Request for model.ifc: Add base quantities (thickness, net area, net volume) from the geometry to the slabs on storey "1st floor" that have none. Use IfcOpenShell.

First a look at what the model holds.

```python
import ifcopenshell
import ifcopenshell.util.element
import ifcopenshell.util.unit

model = ifcopenshell.open("model.ifc")
print(model.schema)
for unit_type in ("LENGTHUNIT", "AREAUNIT", "VOLUMEUNIT"):
    print(unit_type, ifcopenshell.util.unit.calculate_unit_scale(model, unit_type))
storey = next(s for s in model.by_type("IfcBuildingStorey") if s.Name == "1st floor")
slabs = [e for e in ifcopenshell.util.element.get_decomposition(storey) if e.is_a("IfcSlab")]
for e in sorted(slabs, key=lambda e: e.id()):
    print(e.id(), e.is_a(), e.Name, list(ifcopenshell.util.element.get_psets(e, qtos_only=True)), sep=" | ")
```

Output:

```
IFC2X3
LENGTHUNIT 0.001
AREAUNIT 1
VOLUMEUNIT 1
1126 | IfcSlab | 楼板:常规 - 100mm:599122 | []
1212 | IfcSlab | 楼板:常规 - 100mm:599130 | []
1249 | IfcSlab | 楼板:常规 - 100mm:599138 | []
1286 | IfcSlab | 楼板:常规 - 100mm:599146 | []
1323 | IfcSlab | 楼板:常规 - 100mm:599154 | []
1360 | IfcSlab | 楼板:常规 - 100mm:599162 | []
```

```python
import ifcopenshell
import ifcopenshell.api.pset
import ifcopenshell.geom
import ifcopenshell.util.element
import ifcopenshell.util.shape
import ifcopenshell.util.unit

model = ifcopenshell.open("model.ifc")
unit_scale = ifcopenshell.util.unit.calculate_unit_scale(model)
area_scale = ifcopenshell.util.unit.calculate_unit_scale(model, "AREAUNIT")
volume_scale = ifcopenshell.util.unit.calculate_unit_scale(model, "VOLUMEUNIT")
settings = ifcopenshell.geom.settings()

storey = next(s for s in model.by_type("IfcBuildingStorey") if s.Name == "1st floor")
slabs = [e for e in ifcopenshell.util.element.get_decomposition(storey) if e.is_a("IfcSlab")]

for e in sorted(slabs, key=lambda e: e.id()):
    if ifcopenshell.util.element.get_psets(e, qtos_only=True, should_inherit=False):
        continue
    # Geometry comes back in metres, in the element's own axes.
    shape = ifcopenshell.geom.create_shape(settings, e)
    values = {
        "Width": ifcopenshell.util.shape.get_z(shape.geometry) / unit_scale,
        "NetArea": ifcopenshell.util.shape.get_footprint_area(shape.geometry) / area_scale,
        "NetVolume": ifcopenshell.util.shape.get_volume(shape.geometry) / volume_scale,
    }
    qto = ifcopenshell.api.pset.add_qto(model, product=e, name="BaseQuantities")
    ifcopenshell.api.pset.edit_qto(model, qto=qto, properties=values)
    print(e.id(), {k: round(v, 3) for k, v in values.items()})

model.write("model-out.ifc")
```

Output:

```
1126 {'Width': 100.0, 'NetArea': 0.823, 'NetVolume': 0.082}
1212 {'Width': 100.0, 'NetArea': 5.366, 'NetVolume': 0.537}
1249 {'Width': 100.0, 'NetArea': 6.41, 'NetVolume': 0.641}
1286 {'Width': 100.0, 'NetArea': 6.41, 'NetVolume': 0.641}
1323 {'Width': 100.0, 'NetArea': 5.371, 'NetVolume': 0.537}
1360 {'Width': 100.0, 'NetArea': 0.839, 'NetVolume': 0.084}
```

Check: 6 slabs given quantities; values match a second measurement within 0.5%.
